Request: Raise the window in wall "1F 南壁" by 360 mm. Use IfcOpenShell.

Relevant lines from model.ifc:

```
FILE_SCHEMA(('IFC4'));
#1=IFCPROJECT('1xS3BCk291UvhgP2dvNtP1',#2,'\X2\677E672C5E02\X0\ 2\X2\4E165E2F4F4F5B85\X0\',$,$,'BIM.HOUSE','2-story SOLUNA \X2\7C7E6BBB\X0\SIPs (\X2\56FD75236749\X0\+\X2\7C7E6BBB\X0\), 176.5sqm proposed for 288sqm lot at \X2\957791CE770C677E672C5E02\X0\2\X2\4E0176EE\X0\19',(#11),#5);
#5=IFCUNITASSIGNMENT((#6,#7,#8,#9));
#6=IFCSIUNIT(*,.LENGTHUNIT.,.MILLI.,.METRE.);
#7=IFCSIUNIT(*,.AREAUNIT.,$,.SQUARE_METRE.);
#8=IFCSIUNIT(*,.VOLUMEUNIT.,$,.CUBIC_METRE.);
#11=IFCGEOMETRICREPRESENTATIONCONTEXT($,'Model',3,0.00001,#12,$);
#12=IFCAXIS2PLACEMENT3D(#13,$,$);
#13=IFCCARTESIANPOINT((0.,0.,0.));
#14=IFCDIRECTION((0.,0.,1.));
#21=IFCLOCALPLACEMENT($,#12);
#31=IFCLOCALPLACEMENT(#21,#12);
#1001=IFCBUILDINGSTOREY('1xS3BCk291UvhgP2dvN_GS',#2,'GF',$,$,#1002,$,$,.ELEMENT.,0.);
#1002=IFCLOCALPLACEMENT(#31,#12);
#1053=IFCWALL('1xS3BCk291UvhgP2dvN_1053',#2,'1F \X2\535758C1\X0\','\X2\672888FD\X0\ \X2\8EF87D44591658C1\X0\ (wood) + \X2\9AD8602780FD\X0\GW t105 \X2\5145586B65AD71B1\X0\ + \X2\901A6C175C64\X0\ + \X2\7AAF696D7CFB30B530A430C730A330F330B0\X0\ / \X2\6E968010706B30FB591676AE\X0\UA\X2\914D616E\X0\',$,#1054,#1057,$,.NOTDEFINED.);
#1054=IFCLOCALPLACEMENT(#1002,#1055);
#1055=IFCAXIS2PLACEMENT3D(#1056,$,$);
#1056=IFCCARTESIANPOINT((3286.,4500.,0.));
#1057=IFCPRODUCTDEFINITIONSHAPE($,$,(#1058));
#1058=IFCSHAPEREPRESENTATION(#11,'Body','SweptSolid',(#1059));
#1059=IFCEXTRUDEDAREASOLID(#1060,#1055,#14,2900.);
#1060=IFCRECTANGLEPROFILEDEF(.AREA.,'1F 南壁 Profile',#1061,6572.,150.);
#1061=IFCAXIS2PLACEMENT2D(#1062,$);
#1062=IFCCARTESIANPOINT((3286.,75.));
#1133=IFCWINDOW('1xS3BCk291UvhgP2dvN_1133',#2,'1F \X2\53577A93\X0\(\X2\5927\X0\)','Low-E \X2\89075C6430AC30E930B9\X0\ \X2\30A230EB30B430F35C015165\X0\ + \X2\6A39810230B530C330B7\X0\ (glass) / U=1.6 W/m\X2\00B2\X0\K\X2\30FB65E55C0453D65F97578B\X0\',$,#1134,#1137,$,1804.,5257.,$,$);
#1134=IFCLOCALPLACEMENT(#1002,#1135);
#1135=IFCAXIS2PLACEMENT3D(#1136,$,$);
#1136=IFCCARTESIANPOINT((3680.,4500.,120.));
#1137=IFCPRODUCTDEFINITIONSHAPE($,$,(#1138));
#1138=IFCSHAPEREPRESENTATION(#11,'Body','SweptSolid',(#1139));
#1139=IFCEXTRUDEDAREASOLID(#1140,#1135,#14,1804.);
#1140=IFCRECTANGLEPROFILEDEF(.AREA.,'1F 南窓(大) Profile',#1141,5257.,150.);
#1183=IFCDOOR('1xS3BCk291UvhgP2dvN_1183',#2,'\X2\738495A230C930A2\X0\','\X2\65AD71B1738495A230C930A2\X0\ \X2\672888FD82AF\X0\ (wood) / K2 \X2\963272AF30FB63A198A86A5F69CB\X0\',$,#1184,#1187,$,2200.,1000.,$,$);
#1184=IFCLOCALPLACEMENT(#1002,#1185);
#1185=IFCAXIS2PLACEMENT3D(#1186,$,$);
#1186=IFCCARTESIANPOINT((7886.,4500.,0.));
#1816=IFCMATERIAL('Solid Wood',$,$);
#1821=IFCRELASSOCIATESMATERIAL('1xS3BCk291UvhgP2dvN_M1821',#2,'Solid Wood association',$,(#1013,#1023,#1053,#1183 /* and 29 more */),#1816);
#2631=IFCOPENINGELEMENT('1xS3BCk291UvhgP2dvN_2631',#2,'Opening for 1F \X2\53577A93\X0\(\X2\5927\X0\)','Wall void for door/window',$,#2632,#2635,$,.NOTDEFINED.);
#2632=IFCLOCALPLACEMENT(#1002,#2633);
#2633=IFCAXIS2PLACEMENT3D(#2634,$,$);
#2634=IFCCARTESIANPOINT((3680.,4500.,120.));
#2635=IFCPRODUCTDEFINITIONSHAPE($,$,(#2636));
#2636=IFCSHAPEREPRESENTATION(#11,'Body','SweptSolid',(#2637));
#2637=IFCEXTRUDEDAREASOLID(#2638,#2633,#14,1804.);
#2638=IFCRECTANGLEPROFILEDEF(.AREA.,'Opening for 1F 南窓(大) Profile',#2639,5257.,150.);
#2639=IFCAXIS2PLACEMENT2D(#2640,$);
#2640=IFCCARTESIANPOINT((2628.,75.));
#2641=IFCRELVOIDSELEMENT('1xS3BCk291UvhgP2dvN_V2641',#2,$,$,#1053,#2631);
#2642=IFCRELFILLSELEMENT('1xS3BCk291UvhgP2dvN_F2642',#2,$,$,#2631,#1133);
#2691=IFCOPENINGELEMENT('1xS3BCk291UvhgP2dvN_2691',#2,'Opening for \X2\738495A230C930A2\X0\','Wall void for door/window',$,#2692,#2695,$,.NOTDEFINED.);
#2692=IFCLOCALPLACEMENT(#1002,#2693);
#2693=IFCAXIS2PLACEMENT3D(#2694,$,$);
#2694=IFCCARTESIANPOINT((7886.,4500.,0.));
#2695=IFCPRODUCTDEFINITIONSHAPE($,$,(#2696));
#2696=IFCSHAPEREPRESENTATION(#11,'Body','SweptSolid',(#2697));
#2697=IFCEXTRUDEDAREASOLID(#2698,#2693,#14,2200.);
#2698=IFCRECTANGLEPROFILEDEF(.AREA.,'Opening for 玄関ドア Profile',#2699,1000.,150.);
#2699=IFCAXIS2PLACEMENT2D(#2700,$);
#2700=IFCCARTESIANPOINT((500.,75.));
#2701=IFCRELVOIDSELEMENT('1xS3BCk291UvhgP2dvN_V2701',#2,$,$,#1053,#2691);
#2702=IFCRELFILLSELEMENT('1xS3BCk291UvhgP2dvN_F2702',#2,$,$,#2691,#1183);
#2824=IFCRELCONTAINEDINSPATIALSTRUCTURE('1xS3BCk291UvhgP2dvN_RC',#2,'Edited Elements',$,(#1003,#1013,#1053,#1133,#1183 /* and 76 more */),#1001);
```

```python
import numpy as np
import ifcopenshell
import ifcopenshell.api.geometry
import ifcopenshell.util.placement
import ifcopenshell.util.unit

model = ifcopenshell.open("model.ifc")
unit_scale = ifcopenshell.util.unit.calculate_unit_scale(model)

window = model.by_guid("1xS3BCk291UvhgP2dvN_1133")
opening = window.FillsVoids[0].RelatingOpeningElement
dz = 360.0

shift = np.array([0.0, 0.0, dz])
# The window is not placed relative to its opening, so move both.
for product in (opening, window):
    matrix = ifcopenshell.util.placement.get_local_placement(product.ObjectPlacement)
    matrix[:3, 3] += shift
    ifcopenshell.api.geometry.edit_object_placement(model, product=product, matrix=matrix, is_si=False)

print(f"moved by {dz * unit_scale:+.3f} m")

model.write("model_updated.ifc")
```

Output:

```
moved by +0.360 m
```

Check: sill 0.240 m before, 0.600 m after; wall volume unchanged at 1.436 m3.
